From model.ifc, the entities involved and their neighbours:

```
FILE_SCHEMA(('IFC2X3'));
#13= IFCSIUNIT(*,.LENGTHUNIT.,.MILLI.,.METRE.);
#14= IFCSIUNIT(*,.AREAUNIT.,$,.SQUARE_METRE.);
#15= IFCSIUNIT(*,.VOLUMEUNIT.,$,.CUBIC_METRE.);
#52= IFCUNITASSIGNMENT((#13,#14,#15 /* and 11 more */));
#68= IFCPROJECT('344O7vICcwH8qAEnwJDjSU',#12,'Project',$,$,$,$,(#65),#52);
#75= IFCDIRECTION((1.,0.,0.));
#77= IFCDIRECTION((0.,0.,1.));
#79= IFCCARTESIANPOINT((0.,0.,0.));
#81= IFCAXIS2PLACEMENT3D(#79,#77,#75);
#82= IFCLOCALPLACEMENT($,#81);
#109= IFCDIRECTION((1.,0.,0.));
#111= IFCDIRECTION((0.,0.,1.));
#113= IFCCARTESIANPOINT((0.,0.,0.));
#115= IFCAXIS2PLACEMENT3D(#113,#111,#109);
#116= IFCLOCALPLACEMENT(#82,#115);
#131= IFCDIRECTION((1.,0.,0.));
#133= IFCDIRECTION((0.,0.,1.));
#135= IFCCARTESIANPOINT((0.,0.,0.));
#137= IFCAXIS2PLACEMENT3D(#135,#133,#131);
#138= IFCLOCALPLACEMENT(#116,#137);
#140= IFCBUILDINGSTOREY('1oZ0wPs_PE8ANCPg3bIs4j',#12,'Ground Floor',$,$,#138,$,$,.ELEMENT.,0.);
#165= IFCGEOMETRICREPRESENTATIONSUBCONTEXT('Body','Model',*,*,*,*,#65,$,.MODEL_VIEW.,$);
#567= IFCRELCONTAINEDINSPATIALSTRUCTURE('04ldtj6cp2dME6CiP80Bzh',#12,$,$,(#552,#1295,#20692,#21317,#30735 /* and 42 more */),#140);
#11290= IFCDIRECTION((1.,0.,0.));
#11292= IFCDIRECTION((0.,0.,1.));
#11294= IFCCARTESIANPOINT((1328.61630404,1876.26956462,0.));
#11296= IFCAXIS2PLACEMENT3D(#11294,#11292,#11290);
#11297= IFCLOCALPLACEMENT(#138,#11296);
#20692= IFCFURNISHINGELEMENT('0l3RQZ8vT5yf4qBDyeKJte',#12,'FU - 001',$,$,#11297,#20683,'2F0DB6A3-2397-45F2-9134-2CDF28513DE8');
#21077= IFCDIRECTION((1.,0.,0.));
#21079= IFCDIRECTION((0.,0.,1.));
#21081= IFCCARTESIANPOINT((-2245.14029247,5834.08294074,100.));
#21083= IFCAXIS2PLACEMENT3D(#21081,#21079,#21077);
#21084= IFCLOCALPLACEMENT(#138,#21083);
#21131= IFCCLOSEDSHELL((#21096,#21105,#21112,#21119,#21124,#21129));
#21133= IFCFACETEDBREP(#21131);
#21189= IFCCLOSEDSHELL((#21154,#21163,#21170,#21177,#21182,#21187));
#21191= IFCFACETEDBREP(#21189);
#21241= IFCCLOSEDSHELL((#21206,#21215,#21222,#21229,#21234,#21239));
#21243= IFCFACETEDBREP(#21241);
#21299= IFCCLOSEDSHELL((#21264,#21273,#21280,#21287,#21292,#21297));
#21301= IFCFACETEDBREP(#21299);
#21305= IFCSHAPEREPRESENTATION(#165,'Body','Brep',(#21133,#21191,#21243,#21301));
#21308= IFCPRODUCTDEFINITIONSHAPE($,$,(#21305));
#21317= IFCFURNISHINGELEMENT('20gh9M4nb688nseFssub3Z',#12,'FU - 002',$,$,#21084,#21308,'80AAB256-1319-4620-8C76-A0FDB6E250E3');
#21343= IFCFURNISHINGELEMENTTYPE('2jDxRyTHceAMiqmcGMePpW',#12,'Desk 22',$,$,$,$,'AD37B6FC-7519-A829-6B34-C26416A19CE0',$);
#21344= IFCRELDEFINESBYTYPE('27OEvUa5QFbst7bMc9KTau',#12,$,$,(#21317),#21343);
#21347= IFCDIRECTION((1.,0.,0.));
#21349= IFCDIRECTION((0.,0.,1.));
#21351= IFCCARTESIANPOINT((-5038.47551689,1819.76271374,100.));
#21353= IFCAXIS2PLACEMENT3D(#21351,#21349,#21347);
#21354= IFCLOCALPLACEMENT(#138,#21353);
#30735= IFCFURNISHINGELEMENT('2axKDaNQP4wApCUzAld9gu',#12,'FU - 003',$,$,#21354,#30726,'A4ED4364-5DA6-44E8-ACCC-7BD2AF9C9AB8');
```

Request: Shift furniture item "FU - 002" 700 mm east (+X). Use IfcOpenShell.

```python
import ifcopenshell
import ifcopenshell.api.geometry
import ifcopenshell.util.placement
import ifcopenshell.util.unit

model = ifcopenshell.open("model.ifc")
unit_scale = ifcopenshell.util.unit.calculate_unit_scale(model)

item = model.by_guid("20gh9M4nb688nseFssub3Z")
matrix = ifcopenshell.util.placement.get_local_placement(item.ObjectPlacement)
matrix[0, 3] += 0.7 / unit_scale
ifcopenshell.api.geometry.edit_object_placement(model, product=item, matrix=matrix, is_si=False)

print(ifcopenshell.util.placement.get_local_placement(item.ObjectPlacement).round(3) + 0.0)

model.write("model_updated.ifc")
```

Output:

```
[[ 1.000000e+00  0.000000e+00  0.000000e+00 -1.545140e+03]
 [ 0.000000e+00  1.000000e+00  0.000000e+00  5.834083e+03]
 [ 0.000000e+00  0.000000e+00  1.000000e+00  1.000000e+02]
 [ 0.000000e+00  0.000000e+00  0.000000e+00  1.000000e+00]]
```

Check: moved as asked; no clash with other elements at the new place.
